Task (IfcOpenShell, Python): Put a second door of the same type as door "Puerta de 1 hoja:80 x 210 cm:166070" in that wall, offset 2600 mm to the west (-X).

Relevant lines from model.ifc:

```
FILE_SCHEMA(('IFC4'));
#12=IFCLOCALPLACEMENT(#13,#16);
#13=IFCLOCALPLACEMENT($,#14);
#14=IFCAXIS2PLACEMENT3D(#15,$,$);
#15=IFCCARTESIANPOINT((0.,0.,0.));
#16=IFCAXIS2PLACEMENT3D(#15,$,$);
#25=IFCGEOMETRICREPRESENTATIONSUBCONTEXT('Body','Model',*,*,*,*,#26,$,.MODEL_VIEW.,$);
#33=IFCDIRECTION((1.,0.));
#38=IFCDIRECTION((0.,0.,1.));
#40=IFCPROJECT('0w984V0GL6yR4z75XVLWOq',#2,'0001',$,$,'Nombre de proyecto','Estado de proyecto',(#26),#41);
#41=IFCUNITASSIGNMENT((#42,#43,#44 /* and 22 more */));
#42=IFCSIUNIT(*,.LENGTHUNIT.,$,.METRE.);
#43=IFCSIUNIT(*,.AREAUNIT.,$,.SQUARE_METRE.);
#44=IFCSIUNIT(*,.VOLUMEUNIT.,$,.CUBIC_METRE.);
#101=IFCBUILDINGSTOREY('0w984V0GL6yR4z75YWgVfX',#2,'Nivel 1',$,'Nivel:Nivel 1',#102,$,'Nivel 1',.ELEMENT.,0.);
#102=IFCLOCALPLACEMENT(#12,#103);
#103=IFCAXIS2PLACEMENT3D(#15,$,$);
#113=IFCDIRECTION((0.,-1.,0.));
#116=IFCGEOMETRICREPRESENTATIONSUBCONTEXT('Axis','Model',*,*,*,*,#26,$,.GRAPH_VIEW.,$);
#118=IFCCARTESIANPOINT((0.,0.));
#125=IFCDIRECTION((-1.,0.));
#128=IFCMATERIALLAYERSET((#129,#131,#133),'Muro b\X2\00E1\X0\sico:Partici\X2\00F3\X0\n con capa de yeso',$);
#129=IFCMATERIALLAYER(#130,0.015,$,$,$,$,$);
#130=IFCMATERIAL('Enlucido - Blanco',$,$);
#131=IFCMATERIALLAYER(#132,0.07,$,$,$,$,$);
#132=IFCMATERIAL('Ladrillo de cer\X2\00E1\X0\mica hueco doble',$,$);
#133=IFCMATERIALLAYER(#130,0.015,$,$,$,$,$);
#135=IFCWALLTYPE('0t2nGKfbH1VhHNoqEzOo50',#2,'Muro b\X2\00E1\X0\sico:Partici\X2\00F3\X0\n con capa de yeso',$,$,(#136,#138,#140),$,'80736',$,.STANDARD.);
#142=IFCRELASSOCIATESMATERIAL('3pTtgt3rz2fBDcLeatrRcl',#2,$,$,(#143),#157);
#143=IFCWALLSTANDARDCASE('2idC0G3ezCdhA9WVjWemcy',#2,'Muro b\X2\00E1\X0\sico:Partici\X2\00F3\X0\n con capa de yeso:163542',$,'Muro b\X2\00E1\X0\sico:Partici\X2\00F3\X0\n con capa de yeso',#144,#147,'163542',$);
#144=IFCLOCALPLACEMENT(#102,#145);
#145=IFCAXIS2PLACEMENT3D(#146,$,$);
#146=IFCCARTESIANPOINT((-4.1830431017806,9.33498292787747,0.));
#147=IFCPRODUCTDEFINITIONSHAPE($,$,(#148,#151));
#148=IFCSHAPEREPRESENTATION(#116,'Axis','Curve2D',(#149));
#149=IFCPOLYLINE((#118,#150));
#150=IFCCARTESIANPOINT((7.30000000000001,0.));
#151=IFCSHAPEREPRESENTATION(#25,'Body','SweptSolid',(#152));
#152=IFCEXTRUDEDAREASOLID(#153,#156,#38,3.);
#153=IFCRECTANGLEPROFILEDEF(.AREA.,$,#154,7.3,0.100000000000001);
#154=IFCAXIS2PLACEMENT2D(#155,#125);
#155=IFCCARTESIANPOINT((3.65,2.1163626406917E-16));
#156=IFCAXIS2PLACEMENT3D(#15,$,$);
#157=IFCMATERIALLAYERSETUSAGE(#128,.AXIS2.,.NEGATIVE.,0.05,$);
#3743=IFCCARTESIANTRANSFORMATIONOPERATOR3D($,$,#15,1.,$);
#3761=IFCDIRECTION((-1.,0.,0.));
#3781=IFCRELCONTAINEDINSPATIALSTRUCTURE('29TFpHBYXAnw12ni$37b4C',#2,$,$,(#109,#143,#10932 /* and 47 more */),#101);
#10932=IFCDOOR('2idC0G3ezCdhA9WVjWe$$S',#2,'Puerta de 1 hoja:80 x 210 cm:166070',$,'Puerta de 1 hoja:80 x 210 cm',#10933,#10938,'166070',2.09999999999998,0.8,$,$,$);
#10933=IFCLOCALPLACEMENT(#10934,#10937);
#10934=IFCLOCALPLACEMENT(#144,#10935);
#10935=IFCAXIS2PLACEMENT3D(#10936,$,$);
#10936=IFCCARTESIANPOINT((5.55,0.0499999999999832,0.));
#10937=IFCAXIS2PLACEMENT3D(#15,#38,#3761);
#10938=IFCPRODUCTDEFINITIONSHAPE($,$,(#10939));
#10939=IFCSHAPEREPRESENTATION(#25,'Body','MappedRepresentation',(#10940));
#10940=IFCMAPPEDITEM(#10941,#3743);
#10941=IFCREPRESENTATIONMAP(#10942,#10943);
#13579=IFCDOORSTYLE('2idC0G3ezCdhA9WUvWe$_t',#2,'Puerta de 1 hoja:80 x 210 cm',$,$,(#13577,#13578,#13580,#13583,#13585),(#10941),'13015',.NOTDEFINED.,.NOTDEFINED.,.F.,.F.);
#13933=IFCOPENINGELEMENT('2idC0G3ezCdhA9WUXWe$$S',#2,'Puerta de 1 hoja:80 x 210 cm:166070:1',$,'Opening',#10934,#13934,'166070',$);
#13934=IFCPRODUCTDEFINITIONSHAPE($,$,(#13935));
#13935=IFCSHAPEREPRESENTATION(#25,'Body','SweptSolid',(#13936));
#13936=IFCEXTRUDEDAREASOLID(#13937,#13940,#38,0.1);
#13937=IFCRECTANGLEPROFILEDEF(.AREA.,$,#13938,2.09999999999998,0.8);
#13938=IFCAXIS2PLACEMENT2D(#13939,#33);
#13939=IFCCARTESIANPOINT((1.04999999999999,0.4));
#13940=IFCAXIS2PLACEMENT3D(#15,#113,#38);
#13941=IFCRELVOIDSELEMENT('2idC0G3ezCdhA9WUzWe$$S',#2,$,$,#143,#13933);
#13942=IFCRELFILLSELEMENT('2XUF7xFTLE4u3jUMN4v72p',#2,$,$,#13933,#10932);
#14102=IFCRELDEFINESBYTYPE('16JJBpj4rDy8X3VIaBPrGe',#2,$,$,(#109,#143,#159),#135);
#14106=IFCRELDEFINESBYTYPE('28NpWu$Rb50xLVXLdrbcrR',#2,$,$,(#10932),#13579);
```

```python
import ifcopenshell
import ifcopenshell.api.feature
import ifcopenshell.api.geometry
import ifcopenshell.api.root
import ifcopenshell.geom
import ifcopenshell.util.element
import ifcopenshell.util.placement
import ifcopenshell.util.shape
import ifcopenshell.util.unit

model = ifcopenshell.open("model.ifc")
unit_scale = ifcopenshell.util.unit.calculate_unit_scale(model)
settings = ifcopenshell.geom.settings()


def volume(element):
    """Net volume in cubic metres, openings subtracted."""
    shape = ifcopenshell.geom.create_shape(settings, element)
    return ifcopenshell.util.shape.get_volume(shape.geometry)


def reuse_history(source, copy):
    """copy_class also copies each property set's owner history, people and application; keep the originals."""
    for rel in copy.IsDefinedBy:
        if rel.is_a("IfcRelDefinesByProperties") and (history := rel.RelatingPropertyDefinition.OwnerHistory):
            rel.RelatingPropertyDefinition.OwnerHistory = source.OwnerHistory
            ifcopenshell.util.element.remove_deep2(model, history)


door = model.by_id(10932)
opening = door.FillsVoids[0].RelatingOpeningElement
wall = opening.VoidsElements[0].RelatingBuildingElement
before = volume(wall)
shift = ifcopenshell.util.placement.get_local_placement(wall.ObjectPlacement)[:3, 0] * -2.6 / unit_scale

# copy_class copies the void relationship, type, container and properties, but no geometry.
new_opening = ifcopenshell.api.root.copy_class(model, product=opening)
new_opening.Representation = ifcopenshell.util.element.copy_deep(
    model, opening.Representation, exclude=["IfcGeometricRepresentationContext", "IfcRepresentationMap"]
)
new_opening.Name = "Puerta de 1 hoja:80 x 210 cm"
new_opening.Tag = None
new_door = ifcopenshell.api.root.copy_class(model, product=door)
new_door.Representation = ifcopenshell.util.element.copy_deep(
    model, door.Representation, exclude=["IfcGeometricRepresentationContext", "IfcRepresentationMap"]
)
new_door.Name = "Puerta de 1 hoja:80 x 210 cm"
new_door.Tag = None
reuse_history(door, new_door)
ifcopenshell.api.feature.add_filling(model, opening=new_opening, element=new_door)

for old, new in ((opening, new_opening), (door, new_door)):
    matrix = ifcopenshell.util.placement.get_local_placement(old.ObjectPlacement)
    matrix[:3, 3] += shift
    ifcopenshell.api.geometry.edit_object_placement(model, product=new, matrix=matrix, is_si=False)

after = volume(wall)

print(f"wall volume {before:.3f} -> {after:.3f} m3")

model.write("model-out.ifc")
```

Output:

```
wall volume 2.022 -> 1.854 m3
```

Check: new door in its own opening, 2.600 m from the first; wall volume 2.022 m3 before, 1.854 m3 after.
